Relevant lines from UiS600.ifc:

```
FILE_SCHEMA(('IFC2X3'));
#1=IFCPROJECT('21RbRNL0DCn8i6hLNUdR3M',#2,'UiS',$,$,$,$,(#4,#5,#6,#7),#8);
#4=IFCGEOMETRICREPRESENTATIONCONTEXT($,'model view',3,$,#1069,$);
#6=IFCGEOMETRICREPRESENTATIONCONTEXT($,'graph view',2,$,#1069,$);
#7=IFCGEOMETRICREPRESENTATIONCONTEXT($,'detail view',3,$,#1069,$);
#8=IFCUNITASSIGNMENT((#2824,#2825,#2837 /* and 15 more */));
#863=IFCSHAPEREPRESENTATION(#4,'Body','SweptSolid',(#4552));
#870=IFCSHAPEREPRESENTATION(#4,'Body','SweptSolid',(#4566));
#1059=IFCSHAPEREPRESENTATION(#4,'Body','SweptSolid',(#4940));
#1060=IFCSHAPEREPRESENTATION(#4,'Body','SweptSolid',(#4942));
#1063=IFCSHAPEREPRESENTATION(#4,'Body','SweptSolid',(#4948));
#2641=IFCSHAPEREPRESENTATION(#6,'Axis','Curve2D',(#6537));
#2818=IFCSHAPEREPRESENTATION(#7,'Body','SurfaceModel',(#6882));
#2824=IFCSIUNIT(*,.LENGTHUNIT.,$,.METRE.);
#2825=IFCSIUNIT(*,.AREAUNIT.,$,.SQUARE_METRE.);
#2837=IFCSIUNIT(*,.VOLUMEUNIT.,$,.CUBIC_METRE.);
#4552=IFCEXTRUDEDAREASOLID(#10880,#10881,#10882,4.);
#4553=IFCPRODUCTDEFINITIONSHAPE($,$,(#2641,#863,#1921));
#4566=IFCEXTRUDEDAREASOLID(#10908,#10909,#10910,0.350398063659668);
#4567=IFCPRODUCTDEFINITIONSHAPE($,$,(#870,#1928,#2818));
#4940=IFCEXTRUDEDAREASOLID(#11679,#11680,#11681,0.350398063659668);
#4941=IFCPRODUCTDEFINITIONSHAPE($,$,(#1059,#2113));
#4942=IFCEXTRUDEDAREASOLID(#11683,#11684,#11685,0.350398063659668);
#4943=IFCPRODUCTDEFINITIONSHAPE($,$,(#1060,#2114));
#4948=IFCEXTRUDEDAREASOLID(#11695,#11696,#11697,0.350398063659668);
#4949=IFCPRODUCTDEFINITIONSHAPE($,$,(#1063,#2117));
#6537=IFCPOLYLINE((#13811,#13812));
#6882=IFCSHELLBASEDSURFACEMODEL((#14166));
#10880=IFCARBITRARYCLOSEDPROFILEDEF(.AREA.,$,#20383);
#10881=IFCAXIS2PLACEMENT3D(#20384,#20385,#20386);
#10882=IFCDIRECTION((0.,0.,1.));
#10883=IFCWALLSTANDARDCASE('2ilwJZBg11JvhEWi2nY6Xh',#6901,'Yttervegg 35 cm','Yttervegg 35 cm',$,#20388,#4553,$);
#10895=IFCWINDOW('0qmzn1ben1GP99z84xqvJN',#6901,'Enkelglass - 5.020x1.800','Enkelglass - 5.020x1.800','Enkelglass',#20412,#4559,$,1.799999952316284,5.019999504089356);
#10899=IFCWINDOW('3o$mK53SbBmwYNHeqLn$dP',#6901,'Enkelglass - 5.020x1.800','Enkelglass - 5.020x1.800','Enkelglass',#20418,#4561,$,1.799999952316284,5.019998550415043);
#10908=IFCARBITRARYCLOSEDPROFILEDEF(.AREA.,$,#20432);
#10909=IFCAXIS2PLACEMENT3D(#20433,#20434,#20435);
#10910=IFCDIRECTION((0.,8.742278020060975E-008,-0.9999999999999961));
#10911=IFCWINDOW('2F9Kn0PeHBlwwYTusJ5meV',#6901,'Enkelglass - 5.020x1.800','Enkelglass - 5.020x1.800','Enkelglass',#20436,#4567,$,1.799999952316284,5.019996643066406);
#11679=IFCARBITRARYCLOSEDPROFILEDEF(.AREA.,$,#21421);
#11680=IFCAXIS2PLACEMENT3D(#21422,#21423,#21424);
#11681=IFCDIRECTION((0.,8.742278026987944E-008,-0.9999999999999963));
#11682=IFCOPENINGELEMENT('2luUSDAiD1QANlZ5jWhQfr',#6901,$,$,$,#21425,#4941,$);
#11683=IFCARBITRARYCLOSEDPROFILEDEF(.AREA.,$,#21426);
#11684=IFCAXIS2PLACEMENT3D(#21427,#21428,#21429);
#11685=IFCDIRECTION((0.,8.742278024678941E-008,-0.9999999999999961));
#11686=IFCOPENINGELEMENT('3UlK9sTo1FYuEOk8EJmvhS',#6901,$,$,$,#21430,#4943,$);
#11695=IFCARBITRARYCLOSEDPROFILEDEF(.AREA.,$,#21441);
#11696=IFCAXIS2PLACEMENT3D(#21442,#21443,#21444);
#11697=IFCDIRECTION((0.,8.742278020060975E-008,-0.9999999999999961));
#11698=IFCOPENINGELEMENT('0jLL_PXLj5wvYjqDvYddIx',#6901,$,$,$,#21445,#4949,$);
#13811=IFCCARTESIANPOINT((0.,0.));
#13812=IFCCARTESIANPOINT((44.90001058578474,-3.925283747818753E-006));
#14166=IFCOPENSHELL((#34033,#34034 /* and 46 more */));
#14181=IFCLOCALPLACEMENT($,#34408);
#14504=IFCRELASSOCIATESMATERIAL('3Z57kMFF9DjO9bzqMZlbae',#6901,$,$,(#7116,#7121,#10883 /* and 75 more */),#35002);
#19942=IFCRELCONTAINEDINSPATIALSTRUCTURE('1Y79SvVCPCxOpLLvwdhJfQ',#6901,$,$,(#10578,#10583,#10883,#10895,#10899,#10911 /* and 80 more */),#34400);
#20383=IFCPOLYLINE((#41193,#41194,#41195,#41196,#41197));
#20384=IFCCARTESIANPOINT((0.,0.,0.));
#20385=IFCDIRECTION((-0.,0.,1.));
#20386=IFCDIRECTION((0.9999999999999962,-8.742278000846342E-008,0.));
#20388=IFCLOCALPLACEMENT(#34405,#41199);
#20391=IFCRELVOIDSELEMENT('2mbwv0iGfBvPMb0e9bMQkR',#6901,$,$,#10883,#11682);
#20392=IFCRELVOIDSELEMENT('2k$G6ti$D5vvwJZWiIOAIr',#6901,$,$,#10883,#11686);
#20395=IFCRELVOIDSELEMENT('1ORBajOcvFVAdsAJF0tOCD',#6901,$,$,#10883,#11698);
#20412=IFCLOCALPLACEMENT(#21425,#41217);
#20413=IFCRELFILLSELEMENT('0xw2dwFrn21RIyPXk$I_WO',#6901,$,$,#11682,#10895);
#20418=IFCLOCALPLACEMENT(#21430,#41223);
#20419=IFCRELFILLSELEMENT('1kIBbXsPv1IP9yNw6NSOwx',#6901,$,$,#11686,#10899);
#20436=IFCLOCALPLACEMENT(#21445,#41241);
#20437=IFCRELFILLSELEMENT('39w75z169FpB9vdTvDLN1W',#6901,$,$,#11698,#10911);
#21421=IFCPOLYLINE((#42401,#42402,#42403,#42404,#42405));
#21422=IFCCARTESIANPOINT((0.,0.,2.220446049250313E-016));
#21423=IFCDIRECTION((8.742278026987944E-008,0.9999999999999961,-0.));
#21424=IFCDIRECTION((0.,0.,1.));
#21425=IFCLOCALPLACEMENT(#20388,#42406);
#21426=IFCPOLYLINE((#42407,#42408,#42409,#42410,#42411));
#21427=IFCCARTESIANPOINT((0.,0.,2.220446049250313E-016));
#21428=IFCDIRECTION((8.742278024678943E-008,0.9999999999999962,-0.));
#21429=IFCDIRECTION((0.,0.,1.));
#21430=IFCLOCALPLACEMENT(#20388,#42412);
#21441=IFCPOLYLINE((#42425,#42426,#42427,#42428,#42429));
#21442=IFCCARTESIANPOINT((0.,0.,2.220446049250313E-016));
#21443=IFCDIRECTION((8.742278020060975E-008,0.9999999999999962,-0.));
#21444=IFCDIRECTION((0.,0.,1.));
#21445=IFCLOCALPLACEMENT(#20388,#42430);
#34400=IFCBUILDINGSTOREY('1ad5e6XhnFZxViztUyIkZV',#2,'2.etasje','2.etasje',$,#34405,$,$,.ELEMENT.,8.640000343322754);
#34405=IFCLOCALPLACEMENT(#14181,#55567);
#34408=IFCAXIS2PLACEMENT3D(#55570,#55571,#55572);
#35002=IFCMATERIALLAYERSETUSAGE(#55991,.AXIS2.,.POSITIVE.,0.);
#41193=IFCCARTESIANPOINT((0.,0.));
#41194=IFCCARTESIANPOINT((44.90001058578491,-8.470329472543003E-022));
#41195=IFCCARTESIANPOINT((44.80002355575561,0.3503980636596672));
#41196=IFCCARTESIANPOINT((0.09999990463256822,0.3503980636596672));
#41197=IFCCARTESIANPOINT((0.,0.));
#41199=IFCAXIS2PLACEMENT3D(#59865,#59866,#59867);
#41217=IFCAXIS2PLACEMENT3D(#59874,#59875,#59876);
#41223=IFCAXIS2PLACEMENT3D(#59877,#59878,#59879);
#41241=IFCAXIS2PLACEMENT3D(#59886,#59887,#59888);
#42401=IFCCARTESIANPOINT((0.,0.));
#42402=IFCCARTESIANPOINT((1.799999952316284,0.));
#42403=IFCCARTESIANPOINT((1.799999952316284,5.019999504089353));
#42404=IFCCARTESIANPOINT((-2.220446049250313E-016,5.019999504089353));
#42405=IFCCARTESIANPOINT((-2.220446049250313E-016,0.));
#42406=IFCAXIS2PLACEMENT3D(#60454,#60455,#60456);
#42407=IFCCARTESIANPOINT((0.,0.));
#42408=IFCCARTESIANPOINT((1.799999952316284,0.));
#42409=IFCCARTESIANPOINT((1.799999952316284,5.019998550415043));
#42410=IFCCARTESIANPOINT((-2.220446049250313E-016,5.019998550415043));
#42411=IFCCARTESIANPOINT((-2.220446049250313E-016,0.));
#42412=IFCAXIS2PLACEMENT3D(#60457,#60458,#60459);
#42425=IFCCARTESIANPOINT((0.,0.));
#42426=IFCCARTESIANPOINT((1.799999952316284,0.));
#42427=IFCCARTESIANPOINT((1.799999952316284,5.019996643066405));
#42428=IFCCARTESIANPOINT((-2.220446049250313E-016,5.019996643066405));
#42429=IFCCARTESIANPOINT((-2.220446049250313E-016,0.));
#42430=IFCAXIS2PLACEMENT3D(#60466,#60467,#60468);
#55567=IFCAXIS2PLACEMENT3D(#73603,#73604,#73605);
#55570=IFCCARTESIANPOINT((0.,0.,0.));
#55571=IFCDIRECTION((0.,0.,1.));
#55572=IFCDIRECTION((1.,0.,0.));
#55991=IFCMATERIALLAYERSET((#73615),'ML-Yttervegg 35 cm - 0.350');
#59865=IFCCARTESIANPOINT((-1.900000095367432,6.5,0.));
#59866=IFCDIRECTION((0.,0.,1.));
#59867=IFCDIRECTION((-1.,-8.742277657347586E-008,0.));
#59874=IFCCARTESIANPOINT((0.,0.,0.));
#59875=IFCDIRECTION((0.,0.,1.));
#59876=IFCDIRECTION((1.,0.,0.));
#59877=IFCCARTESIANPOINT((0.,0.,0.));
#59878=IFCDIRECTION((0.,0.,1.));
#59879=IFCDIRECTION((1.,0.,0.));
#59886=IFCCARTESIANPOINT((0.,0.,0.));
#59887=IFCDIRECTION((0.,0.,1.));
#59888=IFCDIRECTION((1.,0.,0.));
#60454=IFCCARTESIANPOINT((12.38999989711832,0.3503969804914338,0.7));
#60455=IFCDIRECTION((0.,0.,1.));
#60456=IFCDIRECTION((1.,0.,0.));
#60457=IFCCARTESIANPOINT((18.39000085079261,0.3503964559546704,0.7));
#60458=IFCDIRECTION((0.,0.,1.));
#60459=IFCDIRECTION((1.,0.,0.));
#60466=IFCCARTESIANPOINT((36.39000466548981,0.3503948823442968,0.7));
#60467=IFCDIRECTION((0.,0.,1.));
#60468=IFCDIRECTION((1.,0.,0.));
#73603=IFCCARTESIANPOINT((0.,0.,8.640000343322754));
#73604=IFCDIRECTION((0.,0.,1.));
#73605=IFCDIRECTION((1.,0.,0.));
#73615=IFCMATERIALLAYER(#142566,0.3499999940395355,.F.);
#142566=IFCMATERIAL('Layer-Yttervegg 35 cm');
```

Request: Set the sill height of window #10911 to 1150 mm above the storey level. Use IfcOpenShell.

```python
import numpy as np
import ifcopenshell
import ifcopenshell.api.geometry
import ifcopenshell.geom
import ifcopenshell.util.element
import ifcopenshell.util.placement
import ifcopenshell.util.shape
import ifcopenshell.util.unit

model = ifcopenshell.open("UiS600.ifc")
unit_scale = ifcopenshell.util.unit.calculate_unit_scale(model)

window = model.by_guid("2F9Kn0PeHBlwwYTusJ5meV")
opening = window.FillsVoids[0].RelatingOpeningElement
storey = ifcopenshell.util.element.get_container(window, ifc_class="IfcBuildingStorey")
level = ifcopenshell.util.placement.get_local_placement(storey.ObjectPlacement)[2, 3]

# The opening's origin need not be at the sill, so measure its lowest point.
shape = ifcopenshell.geom.create_shape(ifcopenshell.geom.settings(), opening)
bottom = ifcopenshell.util.shape.get_shape_bottom_elevation(shape, shape.geometry) / unit_scale
dz = level + 1.15 / unit_scale - bottom

shift = np.array([0.0, 0.0, dz])
# The window is placed relative to its opening, so it follows when the opening moves.
matrix = ifcopenshell.util.placement.get_local_placement(opening.ObjectPlacement)
matrix[:3, 3] += shift
ifcopenshell.api.geometry.edit_object_placement(
    model, product=opening, matrix=matrix, is_si=False, should_transform_children=True
)

print(f"moved by {dz * unit_scale:+.3f} m")

model.write("UiS600-out.ifc")
```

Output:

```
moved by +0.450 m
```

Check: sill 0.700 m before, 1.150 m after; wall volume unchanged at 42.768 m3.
